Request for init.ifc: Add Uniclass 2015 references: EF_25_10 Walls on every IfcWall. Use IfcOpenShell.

First a look at what the model holds.

```python
import ifcopenshell

model = ifcopenshell.open("init.ifc")
print(model.schema)
print("classifications:", [c.Name for c in model.by_type("IfcClassification")])
for ifc_class in ("IfcDoor", "IfcRoof", "IfcStair", "IfcWall", "IfcWindow"):
    print(ifc_class, len(model.by_type(ifc_class)))
```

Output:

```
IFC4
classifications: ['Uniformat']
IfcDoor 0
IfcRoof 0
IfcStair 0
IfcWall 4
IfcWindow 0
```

```python
import ifcopenshell
import ifcopenshell.api.classification

model = ifcopenshell.open("init.ifc")

system = ifcopenshell.api.classification.add_classification(model, classification="Uniclass 2015")

codes = {
    "IfcWall": ("EF_25_10", "Walls"),
}
for ifc_class, (code, name) in codes.items():
    products = model.by_type(ifc_class)
    ifcopenshell.api.classification.add_reference(
        model, products=products, classification=system, identification=code, name=name
    )
    print(code, len(products))

model.write("init_updated.ifc")
```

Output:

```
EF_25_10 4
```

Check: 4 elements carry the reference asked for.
